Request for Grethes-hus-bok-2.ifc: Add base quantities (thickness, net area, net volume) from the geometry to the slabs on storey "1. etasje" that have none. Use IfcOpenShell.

First a look at what the model holds.

```python
import ifcopenshell
import ifcopenshell.util.element
import ifcopenshell.util.unit

model = ifcopenshell.open("Grethes-hus-bok-2.ifc")
print(model.schema)
for unit_type in ("LENGTHUNIT", "AREAUNIT", "VOLUMEUNIT"):
    print(unit_type, ifcopenshell.util.unit.calculate_unit_scale(model, unit_type))
storey = next(s for s in model.by_type("IfcBuildingStorey") if s.Name == "1. etasje")
slabs = [e for e in ifcopenshell.util.element.get_decomposition(storey) if e.is_a("IfcSlab")]
for e in sorted(slabs, key=lambda e: e.id()):
    print(e.id(), e.is_a(), e.Name, list(ifcopenshell.util.element.get_psets(e, qtos_only=True)), sep=" | ")
```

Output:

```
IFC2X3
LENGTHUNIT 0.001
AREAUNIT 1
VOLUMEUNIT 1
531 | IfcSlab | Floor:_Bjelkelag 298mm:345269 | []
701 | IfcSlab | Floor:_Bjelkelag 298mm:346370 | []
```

```python
import ifcopenshell
import ifcopenshell.api.pset
import ifcopenshell.geom
import ifcopenshell.util.element
import ifcopenshell.util.shape
import ifcopenshell.util.unit

model = ifcopenshell.open("Grethes-hus-bok-2.ifc")
unit_scale = ifcopenshell.util.unit.calculate_unit_scale(model)
area_scale = ifcopenshell.util.unit.calculate_unit_scale(model, "AREAUNIT")
volume_scale = ifcopenshell.util.unit.calculate_unit_scale(model, "VOLUMEUNIT")
settings = ifcopenshell.geom.settings()

storey = next(s for s in model.by_type("IfcBuildingStorey") if s.Name == "1. etasje")
slabs = [e for e in ifcopenshell.util.element.get_decomposition(storey) if e.is_a("IfcSlab")]

for e in sorted(slabs, key=lambda e: e.id()):
    if ifcopenshell.util.element.get_psets(e, qtos_only=True, should_inherit=False):
        continue
    # Geometry comes back in metres, in the element's own axes.
    shape = ifcopenshell.geom.create_shape(settings, e)
    values = {
        "Width": ifcopenshell.util.shape.get_z(shape.geometry) / unit_scale,
        "NetArea": ifcopenshell.util.shape.get_footprint_area(shape.geometry) / area_scale,
        "NetVolume": ifcopenshell.util.shape.get_volume(shape.geometry) / volume_scale,
    }
    qto = ifcopenshell.api.pset.add_qto(model, product=e, name="BaseQuantities")
    ifcopenshell.api.pset.edit_qto(model, qto=qto, properties=values)
    print(e.id(), {k: round(v, 3) for k, v in values.items()})

model.write("Grethes-hus-bok-2_rev.ifc")
```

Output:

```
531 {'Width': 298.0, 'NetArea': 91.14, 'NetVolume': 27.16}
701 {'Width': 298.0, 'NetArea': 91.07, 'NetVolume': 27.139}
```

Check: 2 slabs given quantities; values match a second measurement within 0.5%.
